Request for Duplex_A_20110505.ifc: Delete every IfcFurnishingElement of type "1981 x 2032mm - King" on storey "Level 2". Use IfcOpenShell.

First a look at what the model holds.

```python
import ifcopenshell
import ifcopenshell.util.element

model = ifcopenshell.open("Duplex_A_20110505.ifc")
print(model.schema)
storey = next(s for s in model.by_type("IfcBuildingStorey") if s.Name == "Level 2")
furniture = [e for e in ifcopenshell.util.element.get_decomposition(storey) if e.is_a("IfcFurnishingElement")]
seen = {}
for e in furniture:
    element_type = ifcopenshell.util.element.get_type(e)
    name = element_type.Name if element_type not in (None, e) else None
    seen[name] = seen.get(name, 0) + 1
for name, count in sorted(seen.items(), key=str):
    print(count, "x", name)
```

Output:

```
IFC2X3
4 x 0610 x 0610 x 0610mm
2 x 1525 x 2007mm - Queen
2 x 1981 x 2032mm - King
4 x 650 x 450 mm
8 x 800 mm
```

```python
import ifcopenshell
import ifcopenshell.api.root
import ifcopenshell.util.element

model = ifcopenshell.open("Duplex_A_20110505.ifc")

storey = next(s for s in model.by_type("IfcBuildingStorey") if s.Name == "Level 2")
furniture = [e for e in ifcopenshell.util.element.get_decomposition(storey) if e.is_a("IfcFurnishingElement")]
targets = [e for e in furniture if (t := ifcopenshell.util.element.get_type(e)) not in (None, e) and t.Name == "1981 x 2032mm - King"]

for e in targets:
    ifcopenshell.api.root.remove_product(model, product=e)
print(len(targets), "removed")

model.write("Duplex_A_20110505-out.ifc")
```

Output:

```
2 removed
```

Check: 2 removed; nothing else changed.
